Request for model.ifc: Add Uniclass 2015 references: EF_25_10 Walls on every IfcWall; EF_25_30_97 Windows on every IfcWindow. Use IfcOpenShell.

First a look at what the model holds.

```python
import ifcopenshell

model = ifcopenshell.open("model.ifc")
print(model.schema)
print("classifications:", [c.Name for c in model.by_type("IfcClassification")])
for ifc_class in ("IfcDoor", "IfcRoof", "IfcStair", "IfcWall", "IfcWindow"):
    print(ifc_class, len(model.by_type(ifc_class)))
```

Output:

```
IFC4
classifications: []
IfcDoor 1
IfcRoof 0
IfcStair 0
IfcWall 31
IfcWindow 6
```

```python
import ifcopenshell
import ifcopenshell.api.classification

model = ifcopenshell.open("model.ifc")

system = ifcopenshell.api.classification.add_classification(model, classification="Uniclass 2015")

codes = {
    "IfcWall": ("EF_25_10", "Walls"),
    "IfcWindow": ("EF_25_30_97", "Windows"),
}
for ifc_class, (code, name) in codes.items():
    products = model.by_type(ifc_class)
    ifcopenshell.api.classification.add_reference(
        model, products=products, classification=system, identification=code, name=name
    )
    print(code, len(products))

model.write("model_edited.ifc")
```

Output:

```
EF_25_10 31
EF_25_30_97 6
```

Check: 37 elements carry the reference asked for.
